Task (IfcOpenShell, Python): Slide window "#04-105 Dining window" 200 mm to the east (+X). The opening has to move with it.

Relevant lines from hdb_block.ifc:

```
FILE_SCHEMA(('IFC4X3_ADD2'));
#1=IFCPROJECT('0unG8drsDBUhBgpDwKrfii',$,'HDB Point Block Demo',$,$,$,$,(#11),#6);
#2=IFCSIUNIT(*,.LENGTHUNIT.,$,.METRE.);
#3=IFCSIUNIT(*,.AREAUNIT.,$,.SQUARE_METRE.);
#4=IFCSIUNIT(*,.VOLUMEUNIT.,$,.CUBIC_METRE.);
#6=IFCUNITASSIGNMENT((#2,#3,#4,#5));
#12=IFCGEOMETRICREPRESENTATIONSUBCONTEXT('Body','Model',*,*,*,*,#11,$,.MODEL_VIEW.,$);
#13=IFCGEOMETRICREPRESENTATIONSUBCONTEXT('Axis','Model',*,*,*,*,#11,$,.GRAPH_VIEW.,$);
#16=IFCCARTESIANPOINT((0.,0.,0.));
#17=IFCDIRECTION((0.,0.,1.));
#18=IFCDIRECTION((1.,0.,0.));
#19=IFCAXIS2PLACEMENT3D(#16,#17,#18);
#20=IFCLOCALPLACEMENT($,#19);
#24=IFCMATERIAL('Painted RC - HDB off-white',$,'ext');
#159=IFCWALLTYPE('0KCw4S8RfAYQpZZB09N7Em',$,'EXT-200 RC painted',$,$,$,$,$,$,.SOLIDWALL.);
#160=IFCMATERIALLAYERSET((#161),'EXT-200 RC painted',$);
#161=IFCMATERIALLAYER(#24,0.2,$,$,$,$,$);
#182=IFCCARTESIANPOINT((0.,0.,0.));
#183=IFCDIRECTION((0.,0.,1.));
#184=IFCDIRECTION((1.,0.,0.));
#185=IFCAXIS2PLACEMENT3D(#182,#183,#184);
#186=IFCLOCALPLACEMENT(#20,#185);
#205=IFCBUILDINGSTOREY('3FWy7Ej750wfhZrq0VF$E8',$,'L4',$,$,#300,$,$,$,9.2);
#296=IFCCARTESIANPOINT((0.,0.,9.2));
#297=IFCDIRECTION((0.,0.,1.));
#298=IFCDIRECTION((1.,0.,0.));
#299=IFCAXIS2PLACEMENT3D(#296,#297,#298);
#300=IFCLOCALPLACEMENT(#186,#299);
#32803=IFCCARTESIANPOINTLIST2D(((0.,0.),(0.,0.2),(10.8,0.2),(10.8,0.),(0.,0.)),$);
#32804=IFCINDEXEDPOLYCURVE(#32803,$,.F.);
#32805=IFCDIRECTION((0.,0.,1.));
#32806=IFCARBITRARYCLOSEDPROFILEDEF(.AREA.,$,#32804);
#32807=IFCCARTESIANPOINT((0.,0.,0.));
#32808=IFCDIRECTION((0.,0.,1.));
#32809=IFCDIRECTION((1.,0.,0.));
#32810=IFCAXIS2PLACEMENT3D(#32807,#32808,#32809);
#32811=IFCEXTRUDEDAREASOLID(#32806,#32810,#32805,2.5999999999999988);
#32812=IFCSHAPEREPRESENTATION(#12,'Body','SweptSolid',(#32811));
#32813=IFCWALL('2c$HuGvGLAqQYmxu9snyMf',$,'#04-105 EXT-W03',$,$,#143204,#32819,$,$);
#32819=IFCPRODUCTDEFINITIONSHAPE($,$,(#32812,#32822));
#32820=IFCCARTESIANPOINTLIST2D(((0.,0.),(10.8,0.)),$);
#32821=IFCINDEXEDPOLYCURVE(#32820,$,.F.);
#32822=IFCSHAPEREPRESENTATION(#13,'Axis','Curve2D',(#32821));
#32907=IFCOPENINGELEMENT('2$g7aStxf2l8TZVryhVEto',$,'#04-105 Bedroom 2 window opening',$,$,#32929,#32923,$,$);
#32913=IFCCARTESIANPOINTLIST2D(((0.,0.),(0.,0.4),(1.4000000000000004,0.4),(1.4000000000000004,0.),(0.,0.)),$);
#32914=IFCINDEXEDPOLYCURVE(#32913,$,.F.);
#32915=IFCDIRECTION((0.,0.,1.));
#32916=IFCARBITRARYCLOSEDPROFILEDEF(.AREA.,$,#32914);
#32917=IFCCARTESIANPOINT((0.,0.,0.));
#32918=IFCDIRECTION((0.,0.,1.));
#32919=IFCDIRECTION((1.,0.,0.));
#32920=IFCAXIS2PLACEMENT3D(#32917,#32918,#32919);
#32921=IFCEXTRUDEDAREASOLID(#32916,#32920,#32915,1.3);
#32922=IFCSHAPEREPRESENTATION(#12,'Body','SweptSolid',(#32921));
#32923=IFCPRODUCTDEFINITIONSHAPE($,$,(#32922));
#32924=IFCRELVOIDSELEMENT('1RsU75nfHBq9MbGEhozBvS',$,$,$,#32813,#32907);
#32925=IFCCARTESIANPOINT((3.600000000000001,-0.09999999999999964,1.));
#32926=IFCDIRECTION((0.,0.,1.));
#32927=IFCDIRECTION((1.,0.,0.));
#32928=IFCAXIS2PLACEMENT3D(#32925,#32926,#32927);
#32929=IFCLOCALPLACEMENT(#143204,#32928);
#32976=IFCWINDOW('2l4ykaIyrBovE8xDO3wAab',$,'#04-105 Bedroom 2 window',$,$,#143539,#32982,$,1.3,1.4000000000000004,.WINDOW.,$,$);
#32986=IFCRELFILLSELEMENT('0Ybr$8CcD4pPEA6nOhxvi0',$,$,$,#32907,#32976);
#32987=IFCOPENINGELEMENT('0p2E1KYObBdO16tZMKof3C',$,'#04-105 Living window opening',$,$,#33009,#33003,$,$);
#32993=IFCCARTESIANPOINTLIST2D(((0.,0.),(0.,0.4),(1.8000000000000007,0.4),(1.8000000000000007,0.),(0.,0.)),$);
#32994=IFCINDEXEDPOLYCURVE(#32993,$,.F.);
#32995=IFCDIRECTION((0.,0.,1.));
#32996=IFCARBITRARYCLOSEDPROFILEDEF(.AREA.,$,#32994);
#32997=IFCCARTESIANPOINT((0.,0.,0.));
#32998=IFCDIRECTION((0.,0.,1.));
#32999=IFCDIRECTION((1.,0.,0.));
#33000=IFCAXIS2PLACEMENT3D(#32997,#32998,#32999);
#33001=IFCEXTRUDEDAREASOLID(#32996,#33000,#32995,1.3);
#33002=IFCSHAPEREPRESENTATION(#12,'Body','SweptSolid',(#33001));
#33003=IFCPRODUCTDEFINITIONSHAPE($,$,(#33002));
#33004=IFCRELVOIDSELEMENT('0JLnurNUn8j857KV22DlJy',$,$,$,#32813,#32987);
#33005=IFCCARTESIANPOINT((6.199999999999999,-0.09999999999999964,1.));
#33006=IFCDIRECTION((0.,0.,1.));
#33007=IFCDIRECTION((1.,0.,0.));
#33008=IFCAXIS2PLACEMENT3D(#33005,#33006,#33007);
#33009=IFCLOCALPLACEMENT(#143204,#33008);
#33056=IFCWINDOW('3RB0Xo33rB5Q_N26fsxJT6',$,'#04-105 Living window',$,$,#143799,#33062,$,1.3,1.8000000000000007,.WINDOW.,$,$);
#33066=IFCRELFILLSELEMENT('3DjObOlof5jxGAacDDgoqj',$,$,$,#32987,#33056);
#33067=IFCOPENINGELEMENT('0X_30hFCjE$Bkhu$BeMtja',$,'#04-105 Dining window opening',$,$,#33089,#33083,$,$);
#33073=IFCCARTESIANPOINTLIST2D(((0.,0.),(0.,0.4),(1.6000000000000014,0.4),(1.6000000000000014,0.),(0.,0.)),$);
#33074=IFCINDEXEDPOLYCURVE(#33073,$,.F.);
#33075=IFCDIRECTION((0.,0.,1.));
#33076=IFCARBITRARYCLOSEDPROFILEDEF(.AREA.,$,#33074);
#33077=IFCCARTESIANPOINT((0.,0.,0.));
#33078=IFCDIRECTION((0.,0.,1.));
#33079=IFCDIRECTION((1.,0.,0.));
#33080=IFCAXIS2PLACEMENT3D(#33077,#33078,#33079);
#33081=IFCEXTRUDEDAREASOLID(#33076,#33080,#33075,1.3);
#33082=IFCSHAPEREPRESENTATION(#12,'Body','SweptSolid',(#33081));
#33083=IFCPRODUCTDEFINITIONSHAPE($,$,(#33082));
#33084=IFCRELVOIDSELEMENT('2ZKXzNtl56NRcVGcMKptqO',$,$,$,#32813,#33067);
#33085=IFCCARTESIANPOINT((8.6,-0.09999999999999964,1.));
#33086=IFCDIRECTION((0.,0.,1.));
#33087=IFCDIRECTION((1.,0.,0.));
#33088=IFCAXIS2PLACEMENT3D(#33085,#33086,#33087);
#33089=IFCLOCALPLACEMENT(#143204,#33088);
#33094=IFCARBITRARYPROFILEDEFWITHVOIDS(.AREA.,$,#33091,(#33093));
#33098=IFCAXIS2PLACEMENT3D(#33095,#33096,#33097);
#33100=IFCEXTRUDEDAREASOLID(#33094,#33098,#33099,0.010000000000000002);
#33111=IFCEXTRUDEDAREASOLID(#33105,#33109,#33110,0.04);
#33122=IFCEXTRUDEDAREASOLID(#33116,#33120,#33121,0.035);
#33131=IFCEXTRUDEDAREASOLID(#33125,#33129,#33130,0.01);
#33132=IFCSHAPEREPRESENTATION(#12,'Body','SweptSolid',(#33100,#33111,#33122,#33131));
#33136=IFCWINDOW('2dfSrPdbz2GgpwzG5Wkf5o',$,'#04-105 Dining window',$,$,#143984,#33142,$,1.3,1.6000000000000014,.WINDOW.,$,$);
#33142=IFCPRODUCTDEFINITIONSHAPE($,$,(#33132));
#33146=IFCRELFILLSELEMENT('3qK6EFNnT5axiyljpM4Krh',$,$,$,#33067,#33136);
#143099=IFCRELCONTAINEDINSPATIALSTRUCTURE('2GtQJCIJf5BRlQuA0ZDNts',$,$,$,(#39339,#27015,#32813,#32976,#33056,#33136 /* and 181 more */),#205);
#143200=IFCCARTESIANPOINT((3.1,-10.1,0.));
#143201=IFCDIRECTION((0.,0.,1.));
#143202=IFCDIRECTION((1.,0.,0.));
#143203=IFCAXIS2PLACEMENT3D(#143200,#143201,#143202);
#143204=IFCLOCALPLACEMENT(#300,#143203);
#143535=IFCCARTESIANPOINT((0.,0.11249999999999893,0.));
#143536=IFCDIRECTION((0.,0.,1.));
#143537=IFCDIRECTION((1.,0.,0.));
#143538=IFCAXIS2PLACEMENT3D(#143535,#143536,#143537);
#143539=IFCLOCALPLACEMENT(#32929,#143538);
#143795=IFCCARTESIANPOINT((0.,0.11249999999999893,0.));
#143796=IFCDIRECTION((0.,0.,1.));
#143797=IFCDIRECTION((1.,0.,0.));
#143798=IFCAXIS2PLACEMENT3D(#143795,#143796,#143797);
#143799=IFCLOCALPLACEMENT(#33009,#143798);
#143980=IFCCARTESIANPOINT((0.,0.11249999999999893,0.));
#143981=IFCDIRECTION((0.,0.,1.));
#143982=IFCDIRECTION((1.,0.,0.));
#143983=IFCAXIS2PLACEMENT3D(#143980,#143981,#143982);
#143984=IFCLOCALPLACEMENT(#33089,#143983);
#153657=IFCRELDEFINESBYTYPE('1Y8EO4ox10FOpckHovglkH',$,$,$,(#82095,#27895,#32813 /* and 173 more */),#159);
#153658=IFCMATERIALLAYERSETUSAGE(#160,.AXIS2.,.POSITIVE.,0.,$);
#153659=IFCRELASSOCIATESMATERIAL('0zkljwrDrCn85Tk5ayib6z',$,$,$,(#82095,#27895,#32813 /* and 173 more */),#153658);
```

```python
import ifcopenshell
import ifcopenshell.api.geometry
import ifcopenshell.util.placement

model = ifcopenshell.open("hdb_block.ifc")

window = model.by_id(33136)
opening = window.FillsVoids[0].RelatingOpeningElement
wall = opening.VoidsElements[0].RelatingBuildingElement

wall_matrix = ifcopenshell.util.placement.get_local_placement(wall.ObjectPlacement)
shift = wall_matrix[:3, 0] * 0.2
before = ifcopenshell.util.placement.get_local_placement(window.ObjectPlacement)[:3, 3].copy()

# The window is placed relative to its opening, so it follows when the opening moves.
matrix = ifcopenshell.util.placement.get_local_placement(opening.ObjectPlacement)
matrix[:3, 3] += shift
ifcopenshell.api.geometry.edit_object_placement(
    model, product=opening, matrix=matrix, is_si=False, should_transform_children=True
)

after = ifcopenshell.util.placement.get_local_placement(window.ObjectPlacement)[:3, 3]
print("window moved by", (after - before).round(3) + 0.0)

model.write("hdb_block_v2.ifc")
```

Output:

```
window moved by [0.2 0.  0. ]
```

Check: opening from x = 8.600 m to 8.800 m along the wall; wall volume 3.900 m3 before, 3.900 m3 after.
